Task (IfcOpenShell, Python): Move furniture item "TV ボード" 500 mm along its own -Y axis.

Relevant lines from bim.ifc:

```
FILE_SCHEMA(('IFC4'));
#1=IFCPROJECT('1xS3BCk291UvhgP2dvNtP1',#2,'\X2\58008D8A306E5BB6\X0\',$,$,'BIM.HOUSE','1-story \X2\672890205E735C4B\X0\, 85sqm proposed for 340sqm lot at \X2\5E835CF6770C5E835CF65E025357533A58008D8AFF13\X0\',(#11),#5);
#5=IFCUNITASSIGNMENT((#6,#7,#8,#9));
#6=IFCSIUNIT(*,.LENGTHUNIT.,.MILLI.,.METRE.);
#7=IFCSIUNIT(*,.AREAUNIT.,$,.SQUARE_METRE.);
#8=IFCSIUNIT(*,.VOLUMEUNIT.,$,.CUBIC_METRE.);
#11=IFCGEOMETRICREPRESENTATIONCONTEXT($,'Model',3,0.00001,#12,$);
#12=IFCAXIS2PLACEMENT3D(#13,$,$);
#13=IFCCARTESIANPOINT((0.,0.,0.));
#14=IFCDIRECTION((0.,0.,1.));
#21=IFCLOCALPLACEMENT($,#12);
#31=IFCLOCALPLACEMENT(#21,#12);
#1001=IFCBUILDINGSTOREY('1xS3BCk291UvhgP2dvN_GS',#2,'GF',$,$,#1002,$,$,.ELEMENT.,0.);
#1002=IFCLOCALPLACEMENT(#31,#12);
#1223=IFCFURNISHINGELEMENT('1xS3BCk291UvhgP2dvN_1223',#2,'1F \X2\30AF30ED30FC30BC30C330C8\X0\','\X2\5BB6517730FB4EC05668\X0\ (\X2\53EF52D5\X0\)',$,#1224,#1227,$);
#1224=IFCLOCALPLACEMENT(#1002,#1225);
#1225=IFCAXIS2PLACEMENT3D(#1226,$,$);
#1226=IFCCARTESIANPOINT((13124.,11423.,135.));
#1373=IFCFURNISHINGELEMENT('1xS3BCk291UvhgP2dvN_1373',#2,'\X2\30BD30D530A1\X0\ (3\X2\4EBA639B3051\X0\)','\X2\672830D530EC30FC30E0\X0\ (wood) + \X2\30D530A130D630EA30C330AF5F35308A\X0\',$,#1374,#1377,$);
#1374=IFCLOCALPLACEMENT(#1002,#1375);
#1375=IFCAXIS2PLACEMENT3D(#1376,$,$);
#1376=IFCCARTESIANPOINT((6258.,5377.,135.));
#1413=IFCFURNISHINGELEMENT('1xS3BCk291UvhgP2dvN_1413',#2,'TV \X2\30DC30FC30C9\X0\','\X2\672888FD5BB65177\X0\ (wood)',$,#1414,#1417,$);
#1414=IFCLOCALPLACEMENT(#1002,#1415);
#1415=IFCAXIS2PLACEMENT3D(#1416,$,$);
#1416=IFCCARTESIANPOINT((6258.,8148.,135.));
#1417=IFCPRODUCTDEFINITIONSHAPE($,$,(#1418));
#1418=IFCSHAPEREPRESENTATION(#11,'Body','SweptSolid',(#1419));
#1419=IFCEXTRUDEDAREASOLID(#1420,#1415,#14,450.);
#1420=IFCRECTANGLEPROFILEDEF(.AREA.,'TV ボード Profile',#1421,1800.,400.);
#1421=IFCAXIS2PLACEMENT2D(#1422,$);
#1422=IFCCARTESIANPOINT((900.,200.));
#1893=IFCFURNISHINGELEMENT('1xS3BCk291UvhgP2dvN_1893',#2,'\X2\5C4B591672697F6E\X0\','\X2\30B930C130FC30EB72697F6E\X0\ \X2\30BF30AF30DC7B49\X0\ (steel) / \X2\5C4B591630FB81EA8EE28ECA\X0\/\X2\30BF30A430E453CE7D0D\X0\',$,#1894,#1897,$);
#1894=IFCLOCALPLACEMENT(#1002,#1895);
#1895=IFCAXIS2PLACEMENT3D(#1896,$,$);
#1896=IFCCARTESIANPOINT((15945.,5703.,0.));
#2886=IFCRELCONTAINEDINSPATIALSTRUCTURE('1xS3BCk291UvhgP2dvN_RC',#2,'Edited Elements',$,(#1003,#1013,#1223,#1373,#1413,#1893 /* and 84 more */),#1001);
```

```python
import ifcopenshell
import ifcopenshell.api.geometry
import ifcopenshell.util.placement
import ifcopenshell.util.unit

model = ifcopenshell.open("bim.ifc")
unit_scale = ifcopenshell.util.unit.calculate_unit_scale(model)

item = model.by_guid("1xS3BCk291UvhgP2dvN_1413")
matrix = ifcopenshell.util.placement.get_local_placement(item.ObjectPlacement)
matrix[:3, 3] -= matrix[:3, 1] * 0.5 / unit_scale
ifcopenshell.api.geometry.edit_object_placement(model, product=item, matrix=matrix, is_si=False)

print(ifcopenshell.util.placement.get_local_placement(item.ObjectPlacement).round(3) + 0.0)

model.write("bim_v2.ifc")
```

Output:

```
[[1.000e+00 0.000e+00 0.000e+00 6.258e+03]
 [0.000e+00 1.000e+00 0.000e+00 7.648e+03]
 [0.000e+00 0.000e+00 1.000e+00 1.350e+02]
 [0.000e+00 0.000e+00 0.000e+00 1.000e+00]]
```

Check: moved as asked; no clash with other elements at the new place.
